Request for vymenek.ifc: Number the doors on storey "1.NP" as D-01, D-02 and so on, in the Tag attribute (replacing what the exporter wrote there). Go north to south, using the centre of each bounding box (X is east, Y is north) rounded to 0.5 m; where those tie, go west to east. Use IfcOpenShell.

First a look at what the model holds.

```python
import ifcopenshell
import ifcopenshell.util.element
import ifcopenshell.util.placement

model = ifcopenshell.open("vymenek.ifc")
print(model.schema)
storey = next(s for s in model.by_type("IfcBuildingStorey") if s.Name == "1.NP")
doors = [e for e in ifcopenshell.util.element.get_decomposition(storey) if e.is_a("IfcDoor")]
for e in sorted(doors, key=lambda e: e.id()):
    origin = ifcopenshell.util.placement.get_local_placement(e.ObjectPlacement)[:3, 3]
    print(e.id(), e.Tag, e.Name, origin.round(2) + 0.0, sep=" | ")
```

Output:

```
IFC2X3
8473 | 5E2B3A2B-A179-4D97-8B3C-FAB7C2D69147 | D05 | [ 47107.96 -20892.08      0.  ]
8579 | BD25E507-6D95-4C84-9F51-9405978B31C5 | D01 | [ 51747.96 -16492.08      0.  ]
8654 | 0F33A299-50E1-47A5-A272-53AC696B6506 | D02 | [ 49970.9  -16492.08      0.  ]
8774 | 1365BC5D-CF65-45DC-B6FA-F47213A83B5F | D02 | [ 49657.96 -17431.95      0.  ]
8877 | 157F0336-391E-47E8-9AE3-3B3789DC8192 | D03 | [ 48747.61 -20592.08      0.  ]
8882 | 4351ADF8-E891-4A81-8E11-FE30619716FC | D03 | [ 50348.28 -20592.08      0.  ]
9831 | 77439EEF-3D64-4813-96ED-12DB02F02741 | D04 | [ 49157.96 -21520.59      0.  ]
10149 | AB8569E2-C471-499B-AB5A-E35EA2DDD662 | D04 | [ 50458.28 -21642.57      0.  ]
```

```python
import ifcopenshell
import ifcopenshell.geom
import ifcopenshell.util.element
import ifcopenshell.util.shape

model = ifcopenshell.open("vymenek.ifc")
settings = ifcopenshell.geom.settings()
settings.set("use-world-coords", True)


def centre(element):
    shape = ifcopenshell.geom.create_shape(settings, element)
    return ifcopenshell.util.shape.get_bbox_centroid(shape.geometry)


storey = next(s for s in model.by_type("IfcBuildingStorey") if s.Name == "1.NP")
doors = [e for e in ifcopenshell.util.element.get_decomposition(storey) if e.is_a("IfcDoor")]

# Insertion points can sit at a corner or the storey origin, so sort by the geometry (in metres).
centres = {e: centre(e) for e in doors}
doors.sort(key=lambda e: (-round(centres[e][1] / 0.5), centres[e][0]))

for i, e in enumerate(doors, start=1):
    number = f"D-{i:02d}"
    e.Tag = number
    print(e.id(), number)

model.write("vymenek_edited.ifc")
```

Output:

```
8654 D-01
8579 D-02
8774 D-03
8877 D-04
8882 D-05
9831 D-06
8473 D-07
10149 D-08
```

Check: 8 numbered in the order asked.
